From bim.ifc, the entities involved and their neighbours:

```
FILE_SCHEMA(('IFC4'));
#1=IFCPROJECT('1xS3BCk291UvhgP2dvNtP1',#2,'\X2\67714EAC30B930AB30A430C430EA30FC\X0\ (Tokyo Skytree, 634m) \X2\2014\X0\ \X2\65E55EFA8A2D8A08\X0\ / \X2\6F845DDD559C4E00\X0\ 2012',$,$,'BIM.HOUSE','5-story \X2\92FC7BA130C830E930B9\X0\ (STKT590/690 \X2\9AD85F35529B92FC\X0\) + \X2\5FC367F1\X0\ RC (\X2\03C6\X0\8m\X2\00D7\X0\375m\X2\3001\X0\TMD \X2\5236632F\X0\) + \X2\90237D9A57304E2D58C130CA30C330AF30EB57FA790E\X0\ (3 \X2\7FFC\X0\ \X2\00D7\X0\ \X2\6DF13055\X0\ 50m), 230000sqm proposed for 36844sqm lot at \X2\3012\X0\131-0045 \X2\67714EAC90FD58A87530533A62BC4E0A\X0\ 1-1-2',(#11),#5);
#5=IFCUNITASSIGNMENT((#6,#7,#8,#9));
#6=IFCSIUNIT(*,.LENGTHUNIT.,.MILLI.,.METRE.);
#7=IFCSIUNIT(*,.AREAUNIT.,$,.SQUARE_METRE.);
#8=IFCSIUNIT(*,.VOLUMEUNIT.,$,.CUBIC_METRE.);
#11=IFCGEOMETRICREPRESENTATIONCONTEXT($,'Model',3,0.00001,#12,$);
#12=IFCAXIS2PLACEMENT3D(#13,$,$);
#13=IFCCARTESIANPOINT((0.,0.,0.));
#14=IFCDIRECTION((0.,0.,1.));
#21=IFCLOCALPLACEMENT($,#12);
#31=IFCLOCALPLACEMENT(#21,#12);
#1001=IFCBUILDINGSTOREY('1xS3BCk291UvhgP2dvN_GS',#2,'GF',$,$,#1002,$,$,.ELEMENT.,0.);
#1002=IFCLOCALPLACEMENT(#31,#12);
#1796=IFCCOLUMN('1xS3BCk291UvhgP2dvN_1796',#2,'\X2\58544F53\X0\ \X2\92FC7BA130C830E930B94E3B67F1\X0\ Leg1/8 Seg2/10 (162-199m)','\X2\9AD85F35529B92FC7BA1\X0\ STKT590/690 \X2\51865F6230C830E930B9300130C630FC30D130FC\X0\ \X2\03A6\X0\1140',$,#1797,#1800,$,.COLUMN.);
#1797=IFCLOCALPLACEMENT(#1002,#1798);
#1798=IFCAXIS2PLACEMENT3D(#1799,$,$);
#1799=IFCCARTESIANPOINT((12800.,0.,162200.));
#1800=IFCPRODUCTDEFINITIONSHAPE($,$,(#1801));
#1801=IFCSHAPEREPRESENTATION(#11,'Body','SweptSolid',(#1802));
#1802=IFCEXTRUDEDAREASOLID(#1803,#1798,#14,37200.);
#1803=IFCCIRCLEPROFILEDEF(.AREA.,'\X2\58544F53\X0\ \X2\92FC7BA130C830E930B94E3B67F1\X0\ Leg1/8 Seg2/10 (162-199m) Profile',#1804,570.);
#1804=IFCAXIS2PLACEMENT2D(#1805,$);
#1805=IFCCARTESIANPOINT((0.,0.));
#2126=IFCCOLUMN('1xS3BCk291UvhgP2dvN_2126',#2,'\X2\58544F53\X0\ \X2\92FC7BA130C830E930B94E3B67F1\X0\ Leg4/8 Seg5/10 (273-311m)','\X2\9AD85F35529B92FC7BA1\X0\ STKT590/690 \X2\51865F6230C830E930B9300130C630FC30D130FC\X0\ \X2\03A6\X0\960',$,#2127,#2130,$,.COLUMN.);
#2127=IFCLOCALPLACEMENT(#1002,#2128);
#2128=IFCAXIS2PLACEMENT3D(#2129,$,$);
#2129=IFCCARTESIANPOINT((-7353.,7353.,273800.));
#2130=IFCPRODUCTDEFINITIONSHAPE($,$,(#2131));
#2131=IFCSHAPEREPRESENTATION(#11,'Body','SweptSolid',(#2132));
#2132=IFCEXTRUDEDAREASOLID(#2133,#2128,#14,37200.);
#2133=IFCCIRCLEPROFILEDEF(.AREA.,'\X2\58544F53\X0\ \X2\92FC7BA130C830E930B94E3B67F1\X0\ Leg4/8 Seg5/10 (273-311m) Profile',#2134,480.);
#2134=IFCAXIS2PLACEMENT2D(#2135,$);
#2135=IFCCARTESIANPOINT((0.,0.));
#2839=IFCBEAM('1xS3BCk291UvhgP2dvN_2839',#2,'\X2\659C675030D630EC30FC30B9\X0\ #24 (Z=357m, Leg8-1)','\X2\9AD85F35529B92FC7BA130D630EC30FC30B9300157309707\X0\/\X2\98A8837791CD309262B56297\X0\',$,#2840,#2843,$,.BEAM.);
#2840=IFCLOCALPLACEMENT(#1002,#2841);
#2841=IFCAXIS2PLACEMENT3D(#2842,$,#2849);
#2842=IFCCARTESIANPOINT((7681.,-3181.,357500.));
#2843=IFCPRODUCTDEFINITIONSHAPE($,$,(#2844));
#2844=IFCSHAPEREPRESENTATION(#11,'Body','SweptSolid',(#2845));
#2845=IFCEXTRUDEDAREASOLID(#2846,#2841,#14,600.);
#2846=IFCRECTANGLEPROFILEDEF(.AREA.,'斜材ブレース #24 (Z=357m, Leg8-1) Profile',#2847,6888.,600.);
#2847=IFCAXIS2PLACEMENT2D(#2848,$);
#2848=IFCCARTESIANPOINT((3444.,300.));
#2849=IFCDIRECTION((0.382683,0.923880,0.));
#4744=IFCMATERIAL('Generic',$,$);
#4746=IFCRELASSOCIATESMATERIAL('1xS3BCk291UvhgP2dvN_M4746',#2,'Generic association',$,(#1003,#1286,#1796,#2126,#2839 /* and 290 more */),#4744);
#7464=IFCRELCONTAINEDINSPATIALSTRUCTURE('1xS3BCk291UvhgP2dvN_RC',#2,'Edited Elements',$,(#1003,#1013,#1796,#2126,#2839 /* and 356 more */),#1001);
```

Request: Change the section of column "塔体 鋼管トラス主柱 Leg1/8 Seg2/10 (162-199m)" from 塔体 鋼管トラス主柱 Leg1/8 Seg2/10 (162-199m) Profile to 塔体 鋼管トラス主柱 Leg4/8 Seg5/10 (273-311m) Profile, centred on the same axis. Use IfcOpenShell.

```python
import ifcopenshell
import ifcopenshell.util.element

model = ifcopenshell.open("bim.ifc")

member = model.by_guid("1xS3BCk291UvhgP2dvN_1796")
source = next(p for p in model.by_type("IfcCircleProfileDef") if p.ProfileName == "塔体 鋼管トラス主柱 Leg4/8 Seg5/10 (273-311m) Profile")

body = next(r for r in member.Representation.Representations if r.RepresentationIdentifier == "Body")
solid = body.Items[0]
old_profile = solid.SweptArea

# Copy the section's sizes but keep this member's own profile position.
profile = ifcopenshell.util.element.copy(model, source)
profile.Position = old_profile.Position
solid.SweptArea = profile
if not model.get_total_inverses(old_profile):
    ifcopenshell.util.element.remove_deep2(model, old_profile)

print(solid.SweptArea)

model.write("bim-out.ifc")
```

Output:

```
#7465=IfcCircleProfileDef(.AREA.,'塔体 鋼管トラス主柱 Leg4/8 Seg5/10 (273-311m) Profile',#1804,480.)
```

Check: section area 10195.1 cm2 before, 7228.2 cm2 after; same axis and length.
